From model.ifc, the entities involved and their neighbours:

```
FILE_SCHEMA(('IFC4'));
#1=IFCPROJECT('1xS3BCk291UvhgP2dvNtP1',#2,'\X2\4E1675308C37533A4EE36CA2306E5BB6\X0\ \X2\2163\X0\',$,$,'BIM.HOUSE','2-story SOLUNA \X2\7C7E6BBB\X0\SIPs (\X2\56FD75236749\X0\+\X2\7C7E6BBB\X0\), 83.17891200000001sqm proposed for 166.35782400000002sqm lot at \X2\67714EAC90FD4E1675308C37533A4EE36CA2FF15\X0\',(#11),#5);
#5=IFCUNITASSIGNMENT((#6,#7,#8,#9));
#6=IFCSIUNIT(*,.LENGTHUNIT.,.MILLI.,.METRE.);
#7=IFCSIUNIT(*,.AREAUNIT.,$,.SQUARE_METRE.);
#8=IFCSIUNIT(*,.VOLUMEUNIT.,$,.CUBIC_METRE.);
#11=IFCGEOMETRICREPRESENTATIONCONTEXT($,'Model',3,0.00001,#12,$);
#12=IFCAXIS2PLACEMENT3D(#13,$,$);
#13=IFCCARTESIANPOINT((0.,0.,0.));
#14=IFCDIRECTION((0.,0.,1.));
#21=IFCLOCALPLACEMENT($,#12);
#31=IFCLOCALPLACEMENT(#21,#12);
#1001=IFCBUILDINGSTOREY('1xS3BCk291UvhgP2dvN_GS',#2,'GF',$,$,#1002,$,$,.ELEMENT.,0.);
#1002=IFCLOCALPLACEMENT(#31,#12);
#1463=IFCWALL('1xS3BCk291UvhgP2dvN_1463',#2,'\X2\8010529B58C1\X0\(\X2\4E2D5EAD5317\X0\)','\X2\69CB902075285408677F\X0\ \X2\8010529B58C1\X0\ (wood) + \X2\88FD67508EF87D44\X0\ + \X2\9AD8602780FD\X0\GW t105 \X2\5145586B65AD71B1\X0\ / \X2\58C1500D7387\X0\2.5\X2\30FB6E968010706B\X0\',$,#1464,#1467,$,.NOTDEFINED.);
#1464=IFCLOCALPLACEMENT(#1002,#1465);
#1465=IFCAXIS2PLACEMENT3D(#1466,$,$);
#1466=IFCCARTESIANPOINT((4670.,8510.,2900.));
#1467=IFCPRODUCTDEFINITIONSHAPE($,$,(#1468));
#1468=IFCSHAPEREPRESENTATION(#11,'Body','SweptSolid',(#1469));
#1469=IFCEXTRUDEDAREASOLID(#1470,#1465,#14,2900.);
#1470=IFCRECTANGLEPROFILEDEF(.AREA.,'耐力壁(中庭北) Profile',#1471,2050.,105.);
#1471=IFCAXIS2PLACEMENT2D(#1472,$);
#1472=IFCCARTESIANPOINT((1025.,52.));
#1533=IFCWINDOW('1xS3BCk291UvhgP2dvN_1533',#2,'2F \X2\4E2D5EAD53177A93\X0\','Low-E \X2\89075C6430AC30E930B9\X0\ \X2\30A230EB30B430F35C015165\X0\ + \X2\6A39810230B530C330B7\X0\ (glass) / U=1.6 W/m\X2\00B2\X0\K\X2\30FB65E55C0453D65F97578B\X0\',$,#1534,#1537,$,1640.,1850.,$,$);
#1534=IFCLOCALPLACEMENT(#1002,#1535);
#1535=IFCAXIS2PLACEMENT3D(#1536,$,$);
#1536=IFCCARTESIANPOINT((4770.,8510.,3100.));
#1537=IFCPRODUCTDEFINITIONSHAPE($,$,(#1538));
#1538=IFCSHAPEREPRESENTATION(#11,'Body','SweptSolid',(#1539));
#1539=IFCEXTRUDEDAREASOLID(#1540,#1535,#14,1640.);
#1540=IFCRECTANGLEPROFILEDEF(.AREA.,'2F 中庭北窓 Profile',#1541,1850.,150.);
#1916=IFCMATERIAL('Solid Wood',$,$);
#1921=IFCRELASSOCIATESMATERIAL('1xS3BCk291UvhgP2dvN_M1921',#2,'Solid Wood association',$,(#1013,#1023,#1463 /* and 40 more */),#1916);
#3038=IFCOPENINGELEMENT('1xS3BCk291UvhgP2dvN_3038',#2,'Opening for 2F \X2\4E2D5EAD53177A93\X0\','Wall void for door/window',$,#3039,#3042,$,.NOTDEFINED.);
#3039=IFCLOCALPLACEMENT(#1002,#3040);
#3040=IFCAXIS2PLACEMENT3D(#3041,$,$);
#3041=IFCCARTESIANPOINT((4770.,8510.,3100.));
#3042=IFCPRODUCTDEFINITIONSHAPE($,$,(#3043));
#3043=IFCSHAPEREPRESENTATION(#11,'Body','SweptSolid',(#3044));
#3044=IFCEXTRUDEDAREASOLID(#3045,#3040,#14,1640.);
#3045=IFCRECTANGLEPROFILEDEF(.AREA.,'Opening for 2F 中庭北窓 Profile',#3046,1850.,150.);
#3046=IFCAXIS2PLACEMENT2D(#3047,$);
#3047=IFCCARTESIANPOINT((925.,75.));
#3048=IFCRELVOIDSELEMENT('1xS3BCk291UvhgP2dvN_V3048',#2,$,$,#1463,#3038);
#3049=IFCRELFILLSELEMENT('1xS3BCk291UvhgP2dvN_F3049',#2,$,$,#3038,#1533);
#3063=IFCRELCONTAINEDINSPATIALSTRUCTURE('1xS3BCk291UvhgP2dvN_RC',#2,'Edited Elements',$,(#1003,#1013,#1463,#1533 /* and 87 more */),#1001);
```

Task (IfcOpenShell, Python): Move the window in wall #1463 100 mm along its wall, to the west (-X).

```python
import ifcopenshell
import ifcopenshell.api.geometry
import ifcopenshell.util.placement
import ifcopenshell.util.unit

model = ifcopenshell.open("model.ifc")
unit_scale = ifcopenshell.util.unit.calculate_unit_scale(model)

window = model.by_guid("1xS3BCk291UvhgP2dvN_1533")
opening = window.FillsVoids[0].RelatingOpeningElement
wall = opening.VoidsElements[0].RelatingBuildingElement

wall_matrix = ifcopenshell.util.placement.get_local_placement(wall.ObjectPlacement)
shift = wall_matrix[:3, 0] * -0.1 / unit_scale
before = ifcopenshell.util.placement.get_local_placement(window.ObjectPlacement)[:3, 3].copy()

# The window is not placed relative to its opening, so move both.
for product in (opening, window):
    matrix = ifcopenshell.util.placement.get_local_placement(product.ObjectPlacement)
    matrix[:3, 3] += shift
    ifcopenshell.api.geometry.edit_object_placement(model, product=product, matrix=matrix, is_si=False)

after = ifcopenshell.util.placement.get_local_placement(window.ObjectPlacement)[:3, 3]
print("window moved by", (after - before).round(3) + 0.0)

model.write("model_updated.ifc")
```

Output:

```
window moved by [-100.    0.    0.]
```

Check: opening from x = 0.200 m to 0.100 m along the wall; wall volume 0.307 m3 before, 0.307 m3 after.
